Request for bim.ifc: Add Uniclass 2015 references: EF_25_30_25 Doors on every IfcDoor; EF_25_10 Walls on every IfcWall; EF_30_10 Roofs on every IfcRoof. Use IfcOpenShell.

First a look at what the model holds.

```python
import ifcopenshell

model = ifcopenshell.open("bim.ifc")
print(model.schema)
print("classifications:", [c.Name for c in model.by_type("IfcClassification")])
for ifc_class in ("IfcDoor", "IfcRoof", "IfcStair", "IfcWall", "IfcWindow"):
    print(ifc_class, len(model.by_type(ifc_class)))
```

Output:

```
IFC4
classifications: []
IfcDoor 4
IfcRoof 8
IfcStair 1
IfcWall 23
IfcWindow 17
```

```python
import ifcopenshell
import ifcopenshell.api.classification

model = ifcopenshell.open("bim.ifc")

system = ifcopenshell.api.classification.add_classification(model, classification="Uniclass 2015")

codes = {
    "IfcDoor": ("EF_25_30_25", "Doors"),
    "IfcWall": ("EF_25_10", "Walls"),
    "IfcRoof": ("EF_30_10", "Roofs"),
}
for ifc_class, (code, name) in codes.items():
    products = model.by_type(ifc_class)
    ifcopenshell.api.classification.add_reference(
        model, products=products, classification=system, identification=code, name=name
    )
    print(code, len(products))

model.write("bim_rev.ifc")
```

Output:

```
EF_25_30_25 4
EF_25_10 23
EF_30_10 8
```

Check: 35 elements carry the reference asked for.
